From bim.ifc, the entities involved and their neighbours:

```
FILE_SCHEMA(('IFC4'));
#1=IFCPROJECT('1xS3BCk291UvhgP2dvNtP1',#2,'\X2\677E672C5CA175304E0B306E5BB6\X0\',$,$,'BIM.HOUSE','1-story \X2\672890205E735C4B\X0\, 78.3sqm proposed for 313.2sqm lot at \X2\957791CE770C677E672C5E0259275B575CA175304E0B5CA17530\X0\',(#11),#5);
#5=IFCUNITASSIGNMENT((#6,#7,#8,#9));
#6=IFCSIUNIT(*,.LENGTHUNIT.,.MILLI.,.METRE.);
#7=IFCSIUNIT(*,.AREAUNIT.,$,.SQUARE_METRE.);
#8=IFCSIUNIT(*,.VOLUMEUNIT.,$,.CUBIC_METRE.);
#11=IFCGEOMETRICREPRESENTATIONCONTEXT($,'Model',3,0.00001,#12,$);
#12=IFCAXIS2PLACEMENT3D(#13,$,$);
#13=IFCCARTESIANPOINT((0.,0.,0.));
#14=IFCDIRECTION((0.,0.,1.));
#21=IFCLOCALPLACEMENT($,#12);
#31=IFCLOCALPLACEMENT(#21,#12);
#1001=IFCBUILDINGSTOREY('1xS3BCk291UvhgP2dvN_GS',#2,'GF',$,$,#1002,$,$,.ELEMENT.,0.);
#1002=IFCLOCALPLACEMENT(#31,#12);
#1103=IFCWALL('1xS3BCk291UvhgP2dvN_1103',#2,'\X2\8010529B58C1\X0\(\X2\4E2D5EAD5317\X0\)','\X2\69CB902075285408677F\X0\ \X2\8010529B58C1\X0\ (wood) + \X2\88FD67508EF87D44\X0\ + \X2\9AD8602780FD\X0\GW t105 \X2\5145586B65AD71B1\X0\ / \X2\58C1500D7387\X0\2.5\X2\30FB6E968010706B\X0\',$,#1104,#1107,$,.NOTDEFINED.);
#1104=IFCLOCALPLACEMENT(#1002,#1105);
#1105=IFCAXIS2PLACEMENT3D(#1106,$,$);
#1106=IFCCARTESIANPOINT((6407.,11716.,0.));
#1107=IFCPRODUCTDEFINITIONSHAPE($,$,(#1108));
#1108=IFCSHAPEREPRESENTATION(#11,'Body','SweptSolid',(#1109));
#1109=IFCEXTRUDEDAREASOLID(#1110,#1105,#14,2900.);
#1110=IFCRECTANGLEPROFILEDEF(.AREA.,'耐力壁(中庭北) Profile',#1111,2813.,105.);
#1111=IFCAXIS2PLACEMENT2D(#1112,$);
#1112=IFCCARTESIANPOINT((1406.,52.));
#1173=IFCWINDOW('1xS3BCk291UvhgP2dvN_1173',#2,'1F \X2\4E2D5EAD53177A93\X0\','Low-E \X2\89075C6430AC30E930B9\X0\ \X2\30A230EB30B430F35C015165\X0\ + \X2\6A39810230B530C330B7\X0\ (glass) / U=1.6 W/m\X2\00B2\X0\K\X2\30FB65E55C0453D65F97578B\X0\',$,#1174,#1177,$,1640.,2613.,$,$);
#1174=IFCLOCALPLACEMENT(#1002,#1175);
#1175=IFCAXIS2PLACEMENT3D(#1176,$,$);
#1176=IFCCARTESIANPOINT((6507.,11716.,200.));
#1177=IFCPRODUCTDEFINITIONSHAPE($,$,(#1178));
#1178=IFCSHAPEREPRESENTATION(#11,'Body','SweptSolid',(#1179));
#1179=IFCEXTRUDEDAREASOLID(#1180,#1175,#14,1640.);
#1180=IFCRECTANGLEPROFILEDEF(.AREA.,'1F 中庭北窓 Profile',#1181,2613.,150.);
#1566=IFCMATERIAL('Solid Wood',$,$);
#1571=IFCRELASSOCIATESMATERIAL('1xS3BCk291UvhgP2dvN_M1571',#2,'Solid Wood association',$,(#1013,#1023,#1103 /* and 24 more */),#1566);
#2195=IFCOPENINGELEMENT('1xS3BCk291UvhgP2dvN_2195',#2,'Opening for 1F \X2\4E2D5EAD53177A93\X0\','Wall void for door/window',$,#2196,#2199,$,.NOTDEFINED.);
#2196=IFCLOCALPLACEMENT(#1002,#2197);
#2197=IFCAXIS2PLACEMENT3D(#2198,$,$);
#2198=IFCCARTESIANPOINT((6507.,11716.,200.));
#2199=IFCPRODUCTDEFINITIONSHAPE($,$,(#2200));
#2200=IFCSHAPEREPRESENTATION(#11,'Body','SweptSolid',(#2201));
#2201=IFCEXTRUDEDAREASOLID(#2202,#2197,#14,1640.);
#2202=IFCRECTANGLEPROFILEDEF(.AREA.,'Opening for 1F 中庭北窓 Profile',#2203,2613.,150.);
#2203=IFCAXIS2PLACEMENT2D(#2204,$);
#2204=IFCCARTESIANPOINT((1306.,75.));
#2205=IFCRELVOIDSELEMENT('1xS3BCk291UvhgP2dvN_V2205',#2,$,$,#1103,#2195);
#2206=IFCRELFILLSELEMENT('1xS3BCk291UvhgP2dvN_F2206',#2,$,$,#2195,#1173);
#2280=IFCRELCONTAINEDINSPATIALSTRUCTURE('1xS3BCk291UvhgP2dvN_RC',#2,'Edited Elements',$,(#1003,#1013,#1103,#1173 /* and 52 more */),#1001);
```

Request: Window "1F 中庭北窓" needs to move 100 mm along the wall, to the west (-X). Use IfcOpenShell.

```python
import ifcopenshell
import ifcopenshell.api.geometry
import ifcopenshell.util.placement
import ifcopenshell.util.unit

model = ifcopenshell.open("bim.ifc")
unit_scale = ifcopenshell.util.unit.calculate_unit_scale(model)

window = model.by_guid("1xS3BCk291UvhgP2dvN_1173")
opening = window.FillsVoids[0].RelatingOpeningElement
wall = opening.VoidsElements[0].RelatingBuildingElement

wall_matrix = ifcopenshell.util.placement.get_local_placement(wall.ObjectPlacement)
shift = wall_matrix[:3, 0] * -0.1 / unit_scale
before = ifcopenshell.util.placement.get_local_placement(window.ObjectPlacement)[:3, 3].copy()

# The window is not placed relative to its opening, so move both.
for product in (opening, window):
    matrix = ifcopenshell.util.placement.get_local_placement(product.ObjectPlacement)
    matrix[:3, 3] += shift
    ifcopenshell.api.geometry.edit_object_placement(model, product=product, matrix=matrix, is_si=False)

after = ifcopenshell.util.placement.get_local_placement(window.ObjectPlacement)[:3, 3]
print("window moved by", (after - before).round(3) + 0.0)

model.write("bim-out.ifc")
```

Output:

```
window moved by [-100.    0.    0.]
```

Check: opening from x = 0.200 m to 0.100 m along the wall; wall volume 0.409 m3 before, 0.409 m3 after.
